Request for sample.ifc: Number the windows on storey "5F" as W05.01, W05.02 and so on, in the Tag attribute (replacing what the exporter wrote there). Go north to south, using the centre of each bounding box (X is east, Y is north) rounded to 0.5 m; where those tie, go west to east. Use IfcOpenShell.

First a look at what the model holds.

```python
import ifcopenshell
import ifcopenshell.util.element
import ifcopenshell.util.placement

model = ifcopenshell.open("sample.ifc")
print(model.schema)
storey = next(s for s in model.by_type("IfcBuildingStorey") if s.Name == "5F")
windows = [e for e in ifcopenshell.util.element.get_decomposition(storey) if e.is_a("IfcWindow")]
for e in sorted(windows, key=lambda e: e.id()):
    origin = ifcopenshell.util.placement.get_local_placement(e.ObjectPlacement)[:3, 3]
    print(e.id(), e.Tag, e.Name, origin.round(2) + 0.0, sep=" | ")
```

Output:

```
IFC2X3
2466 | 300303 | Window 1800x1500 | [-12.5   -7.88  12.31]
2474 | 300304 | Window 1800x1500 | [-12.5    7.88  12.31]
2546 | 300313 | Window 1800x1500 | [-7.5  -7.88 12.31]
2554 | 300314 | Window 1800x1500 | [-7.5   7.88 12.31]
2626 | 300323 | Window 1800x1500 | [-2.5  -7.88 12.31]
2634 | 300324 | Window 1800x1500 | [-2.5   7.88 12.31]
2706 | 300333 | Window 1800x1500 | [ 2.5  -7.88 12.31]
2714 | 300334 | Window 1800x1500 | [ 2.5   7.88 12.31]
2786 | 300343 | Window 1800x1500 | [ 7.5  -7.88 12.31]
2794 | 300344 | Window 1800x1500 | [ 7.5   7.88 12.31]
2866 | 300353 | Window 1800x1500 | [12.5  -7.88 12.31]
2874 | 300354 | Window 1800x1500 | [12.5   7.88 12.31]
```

```python
import ifcopenshell
import ifcopenshell.geom
import ifcopenshell.util.element
import ifcopenshell.util.shape

model = ifcopenshell.open("sample.ifc")
settings = ifcopenshell.geom.settings()
settings.set("use-world-coords", True)


def centre(element):
    shape = ifcopenshell.geom.create_shape(settings, element)
    return ifcopenshell.util.shape.get_bbox_centroid(shape.geometry)


storey = next(s for s in model.by_type("IfcBuildingStorey") if s.Name == "5F")
windows = [e for e in ifcopenshell.util.element.get_decomposition(storey) if e.is_a("IfcWindow")]

# Insertion points can sit at a corner or the storey origin, so sort by the geometry (in metres).
centres = {e: centre(e) for e in windows}
windows.sort(key=lambda e: (-round(centres[e][1] / 0.5), centres[e][0]))

for i, e in enumerate(windows, start=1):
    number = f"W05.{i:02d}"
    e.Tag = number
    print(e.id(), number)

model.write("sample_rev.ifc")
```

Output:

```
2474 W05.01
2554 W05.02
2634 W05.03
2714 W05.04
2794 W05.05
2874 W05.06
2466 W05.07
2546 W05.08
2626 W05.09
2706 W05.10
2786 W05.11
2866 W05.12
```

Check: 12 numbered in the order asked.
